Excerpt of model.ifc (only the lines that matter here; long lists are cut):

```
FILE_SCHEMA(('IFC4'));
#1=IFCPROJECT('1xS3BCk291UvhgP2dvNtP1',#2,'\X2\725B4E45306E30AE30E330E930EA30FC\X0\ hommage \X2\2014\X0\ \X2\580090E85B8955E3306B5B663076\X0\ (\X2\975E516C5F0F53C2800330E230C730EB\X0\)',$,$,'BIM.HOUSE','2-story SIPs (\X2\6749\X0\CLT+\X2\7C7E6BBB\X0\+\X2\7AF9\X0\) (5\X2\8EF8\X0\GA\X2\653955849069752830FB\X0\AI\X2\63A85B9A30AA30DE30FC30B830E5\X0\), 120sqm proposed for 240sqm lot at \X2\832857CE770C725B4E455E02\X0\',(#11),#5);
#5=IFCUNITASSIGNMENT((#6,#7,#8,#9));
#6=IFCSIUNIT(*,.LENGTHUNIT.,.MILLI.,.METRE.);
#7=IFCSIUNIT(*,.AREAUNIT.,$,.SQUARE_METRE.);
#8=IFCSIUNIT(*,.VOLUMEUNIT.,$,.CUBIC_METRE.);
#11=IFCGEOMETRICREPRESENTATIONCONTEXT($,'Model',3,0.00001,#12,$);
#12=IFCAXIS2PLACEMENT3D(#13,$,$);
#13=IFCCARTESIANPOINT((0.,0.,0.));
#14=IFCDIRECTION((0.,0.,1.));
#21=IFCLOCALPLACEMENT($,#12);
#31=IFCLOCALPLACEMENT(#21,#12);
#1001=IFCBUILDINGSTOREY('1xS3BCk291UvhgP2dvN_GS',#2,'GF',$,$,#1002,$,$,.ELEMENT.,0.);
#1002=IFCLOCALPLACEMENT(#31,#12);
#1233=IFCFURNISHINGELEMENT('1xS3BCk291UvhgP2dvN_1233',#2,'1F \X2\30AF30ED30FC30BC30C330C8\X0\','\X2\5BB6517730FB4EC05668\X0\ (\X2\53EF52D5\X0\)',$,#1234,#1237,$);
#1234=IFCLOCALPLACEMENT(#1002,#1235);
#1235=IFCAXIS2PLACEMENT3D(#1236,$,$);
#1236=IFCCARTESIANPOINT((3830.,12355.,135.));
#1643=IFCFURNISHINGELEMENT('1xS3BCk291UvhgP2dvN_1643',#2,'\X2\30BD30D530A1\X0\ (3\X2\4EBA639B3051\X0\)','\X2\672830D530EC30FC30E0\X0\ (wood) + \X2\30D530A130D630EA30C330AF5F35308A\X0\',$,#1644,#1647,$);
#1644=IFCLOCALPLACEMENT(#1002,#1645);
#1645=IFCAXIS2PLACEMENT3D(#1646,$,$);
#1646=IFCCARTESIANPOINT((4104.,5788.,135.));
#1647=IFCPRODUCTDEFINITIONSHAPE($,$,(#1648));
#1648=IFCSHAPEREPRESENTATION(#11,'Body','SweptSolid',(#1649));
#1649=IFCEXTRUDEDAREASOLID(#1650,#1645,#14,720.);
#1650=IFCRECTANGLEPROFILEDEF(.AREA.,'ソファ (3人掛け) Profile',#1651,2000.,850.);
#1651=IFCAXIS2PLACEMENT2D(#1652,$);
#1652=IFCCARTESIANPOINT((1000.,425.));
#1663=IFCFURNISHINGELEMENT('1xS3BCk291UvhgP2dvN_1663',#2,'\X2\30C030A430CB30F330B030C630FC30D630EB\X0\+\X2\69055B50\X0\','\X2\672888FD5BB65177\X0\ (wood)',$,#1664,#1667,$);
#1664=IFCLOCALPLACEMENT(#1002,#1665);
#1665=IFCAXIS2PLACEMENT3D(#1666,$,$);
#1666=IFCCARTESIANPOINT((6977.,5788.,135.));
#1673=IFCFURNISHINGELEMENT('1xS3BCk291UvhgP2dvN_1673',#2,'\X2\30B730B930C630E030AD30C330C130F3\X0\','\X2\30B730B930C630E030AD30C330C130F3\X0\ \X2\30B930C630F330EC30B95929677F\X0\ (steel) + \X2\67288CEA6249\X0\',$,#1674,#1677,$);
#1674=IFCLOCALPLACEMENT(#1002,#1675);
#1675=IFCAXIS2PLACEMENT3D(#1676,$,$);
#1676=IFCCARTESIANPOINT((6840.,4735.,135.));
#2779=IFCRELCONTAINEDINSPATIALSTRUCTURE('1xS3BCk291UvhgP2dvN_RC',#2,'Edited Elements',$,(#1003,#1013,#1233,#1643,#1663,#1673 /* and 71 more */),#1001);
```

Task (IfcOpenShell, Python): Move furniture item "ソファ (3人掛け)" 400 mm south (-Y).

```python
import ifcopenshell
import ifcopenshell.api.geometry
import ifcopenshell.util.placement
import ifcopenshell.util.unit

model = ifcopenshell.open("model.ifc")
unit_scale = ifcopenshell.util.unit.calculate_unit_scale(model)

item = model.by_guid("1xS3BCk291UvhgP2dvN_1643")
matrix = ifcopenshell.util.placement.get_local_placement(item.ObjectPlacement)
matrix[1, 3] -= 0.4 / unit_scale
ifcopenshell.api.geometry.edit_object_placement(model, product=item, matrix=matrix, is_si=False)

print(ifcopenshell.util.placement.get_local_placement(item.ObjectPlacement).round(3) + 0.0)

model.write("model-out.ifc")
```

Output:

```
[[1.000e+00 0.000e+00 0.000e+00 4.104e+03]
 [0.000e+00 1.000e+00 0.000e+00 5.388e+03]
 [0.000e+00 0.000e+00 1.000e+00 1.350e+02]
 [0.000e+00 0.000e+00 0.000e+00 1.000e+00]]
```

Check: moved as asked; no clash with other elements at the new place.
